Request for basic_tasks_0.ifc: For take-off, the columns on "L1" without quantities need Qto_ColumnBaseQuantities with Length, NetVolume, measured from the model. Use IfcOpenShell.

First a look at what the model holds.

```python
import ifcopenshell
import ifcopenshell.util.element
import ifcopenshell.util.unit

model = ifcopenshell.open("basic_tasks_0.ifc")
print(model.schema)
for unit_type in ("LENGTHUNIT", "AREAUNIT", "VOLUMEUNIT"):
    print(unit_type, ifcopenshell.util.unit.calculate_unit_scale(model, unit_type))
storey = next(s for s in model.by_type("IfcBuildingStorey") if s.Name == "L1")
columns = [e for e in ifcopenshell.util.element.get_decomposition(storey) if e.is_a("IfcColumn")]
for e in sorted(columns, key=lambda e: e.id()):
    print(e.id(), e.is_a(), e.Name, list(ifcopenshell.util.element.get_psets(e, qtos_only=True)), sep=" | ")
```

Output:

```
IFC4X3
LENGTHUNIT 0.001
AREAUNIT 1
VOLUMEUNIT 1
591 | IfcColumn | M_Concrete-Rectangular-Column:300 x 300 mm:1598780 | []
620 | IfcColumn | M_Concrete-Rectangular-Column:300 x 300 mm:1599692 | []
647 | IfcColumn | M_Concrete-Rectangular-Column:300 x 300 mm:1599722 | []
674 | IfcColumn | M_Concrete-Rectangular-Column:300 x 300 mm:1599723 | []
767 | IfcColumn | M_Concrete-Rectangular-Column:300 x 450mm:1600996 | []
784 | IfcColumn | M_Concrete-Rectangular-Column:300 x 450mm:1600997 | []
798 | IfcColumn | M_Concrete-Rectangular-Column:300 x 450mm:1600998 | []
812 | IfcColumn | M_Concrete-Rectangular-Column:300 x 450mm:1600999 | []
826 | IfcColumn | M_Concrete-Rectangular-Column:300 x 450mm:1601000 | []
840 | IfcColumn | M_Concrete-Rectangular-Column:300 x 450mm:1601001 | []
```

```python
import ifcopenshell
import ifcopenshell.api.pset
import ifcopenshell.geom
import ifcopenshell.util.element
import ifcopenshell.util.shape
import ifcopenshell.util.unit

model = ifcopenshell.open("basic_tasks_0.ifc")
unit_scale = ifcopenshell.util.unit.calculate_unit_scale(model)
volume_scale = ifcopenshell.util.unit.calculate_unit_scale(model, "VOLUMEUNIT")
settings = ifcopenshell.geom.settings()

storey = next(s for s in model.by_type("IfcBuildingStorey") if s.Name == "L1")
columns = [e for e in ifcopenshell.util.element.get_decomposition(storey) if e.is_a("IfcColumn")]

for e in sorted(columns, key=lambda e: e.id()):
    if ifcopenshell.util.element.get_psets(e, qtos_only=True, should_inherit=False):
        continue
    # Geometry comes back in metres, in the element's own axes.
    shape = ifcopenshell.geom.create_shape(settings, e)
    values = {
        "Length": ifcopenshell.util.shape.get_z(shape.geometry) / unit_scale,
        "NetVolume": ifcopenshell.util.shape.get_volume(shape.geometry) / volume_scale,
    }
    qto = ifcopenshell.api.pset.add_qto(model, product=e, name="Qto_ColumnBaseQuantities")
    ifcopenshell.api.pset.edit_qto(model, qto=qto, properties=values)
    print(e.id(), {k: round(v, 3) for k, v in values.items()})

model.write("basic_tasks_0_edited.ifc")
```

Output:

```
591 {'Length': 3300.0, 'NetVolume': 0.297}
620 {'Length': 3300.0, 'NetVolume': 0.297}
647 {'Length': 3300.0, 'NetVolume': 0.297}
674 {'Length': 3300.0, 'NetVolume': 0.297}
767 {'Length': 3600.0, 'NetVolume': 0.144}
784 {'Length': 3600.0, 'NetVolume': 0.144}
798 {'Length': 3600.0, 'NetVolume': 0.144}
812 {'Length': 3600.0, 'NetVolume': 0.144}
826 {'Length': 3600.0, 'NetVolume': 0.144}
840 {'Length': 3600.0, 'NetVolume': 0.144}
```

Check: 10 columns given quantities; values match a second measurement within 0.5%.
